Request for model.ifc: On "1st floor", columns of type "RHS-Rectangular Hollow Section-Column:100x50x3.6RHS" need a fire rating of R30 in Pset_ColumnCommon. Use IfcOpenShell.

First a look at what the model holds.

```python
import ifcopenshell
import ifcopenshell.util.element

model = ifcopenshell.open("model.ifc")
print(model.schema)
storey = next(s for s in model.by_type("IfcBuildingStorey") if s.Name == "1st floor")
columns = [e for e in ifcopenshell.util.element.get_decomposition(storey) if e.is_a("IfcColumn")]
seen = {}
for e in columns:
    element_type = ifcopenshell.util.element.get_type(e)
    key = (element_type.Name if element_type != e and element_type else None, ifcopenshell.util.element.get_pset(e, "Pset_ColumnCommon", "FireRating"))
    seen[key] = seen.get(key, 0) + 1
for (name, value), count in sorted(seen.items(), key=str):
    print(count, "x", name, "|", value)
```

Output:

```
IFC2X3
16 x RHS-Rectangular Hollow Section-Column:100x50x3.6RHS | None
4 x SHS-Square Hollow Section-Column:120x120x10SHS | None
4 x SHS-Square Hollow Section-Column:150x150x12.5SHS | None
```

```python
import ifcopenshell
import ifcopenshell.api.pset
import ifcopenshell.util.element

model = ifcopenshell.open("model.ifc")

storey = next(s for s in model.by_type("IfcBuildingStorey") if s.Name == "1st floor")
columns = [e for e in ifcopenshell.util.element.get_decomposition(storey) if e.is_a("IfcColumn")]

count = 0
for e in columns:
    element_type = ifcopenshell.util.element.get_type(e)
    if element_type in (None, e) or element_type.Name != "RHS-Rectangular Hollow Section-Column:100x50x3.6RHS":
        continue
    # add_pset returns the element's existing set when there is one.
    pset = ifcopenshell.api.pset.add_pset(model, product=e, name="Pset_ColumnCommon")
    ifcopenshell.api.pset.edit_pset(model, pset=pset, properties={"FireRating": "R30"})
    count += 1

print(count, "columns updated")

model.write("model_updated.ifc")
```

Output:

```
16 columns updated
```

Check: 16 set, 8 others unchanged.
